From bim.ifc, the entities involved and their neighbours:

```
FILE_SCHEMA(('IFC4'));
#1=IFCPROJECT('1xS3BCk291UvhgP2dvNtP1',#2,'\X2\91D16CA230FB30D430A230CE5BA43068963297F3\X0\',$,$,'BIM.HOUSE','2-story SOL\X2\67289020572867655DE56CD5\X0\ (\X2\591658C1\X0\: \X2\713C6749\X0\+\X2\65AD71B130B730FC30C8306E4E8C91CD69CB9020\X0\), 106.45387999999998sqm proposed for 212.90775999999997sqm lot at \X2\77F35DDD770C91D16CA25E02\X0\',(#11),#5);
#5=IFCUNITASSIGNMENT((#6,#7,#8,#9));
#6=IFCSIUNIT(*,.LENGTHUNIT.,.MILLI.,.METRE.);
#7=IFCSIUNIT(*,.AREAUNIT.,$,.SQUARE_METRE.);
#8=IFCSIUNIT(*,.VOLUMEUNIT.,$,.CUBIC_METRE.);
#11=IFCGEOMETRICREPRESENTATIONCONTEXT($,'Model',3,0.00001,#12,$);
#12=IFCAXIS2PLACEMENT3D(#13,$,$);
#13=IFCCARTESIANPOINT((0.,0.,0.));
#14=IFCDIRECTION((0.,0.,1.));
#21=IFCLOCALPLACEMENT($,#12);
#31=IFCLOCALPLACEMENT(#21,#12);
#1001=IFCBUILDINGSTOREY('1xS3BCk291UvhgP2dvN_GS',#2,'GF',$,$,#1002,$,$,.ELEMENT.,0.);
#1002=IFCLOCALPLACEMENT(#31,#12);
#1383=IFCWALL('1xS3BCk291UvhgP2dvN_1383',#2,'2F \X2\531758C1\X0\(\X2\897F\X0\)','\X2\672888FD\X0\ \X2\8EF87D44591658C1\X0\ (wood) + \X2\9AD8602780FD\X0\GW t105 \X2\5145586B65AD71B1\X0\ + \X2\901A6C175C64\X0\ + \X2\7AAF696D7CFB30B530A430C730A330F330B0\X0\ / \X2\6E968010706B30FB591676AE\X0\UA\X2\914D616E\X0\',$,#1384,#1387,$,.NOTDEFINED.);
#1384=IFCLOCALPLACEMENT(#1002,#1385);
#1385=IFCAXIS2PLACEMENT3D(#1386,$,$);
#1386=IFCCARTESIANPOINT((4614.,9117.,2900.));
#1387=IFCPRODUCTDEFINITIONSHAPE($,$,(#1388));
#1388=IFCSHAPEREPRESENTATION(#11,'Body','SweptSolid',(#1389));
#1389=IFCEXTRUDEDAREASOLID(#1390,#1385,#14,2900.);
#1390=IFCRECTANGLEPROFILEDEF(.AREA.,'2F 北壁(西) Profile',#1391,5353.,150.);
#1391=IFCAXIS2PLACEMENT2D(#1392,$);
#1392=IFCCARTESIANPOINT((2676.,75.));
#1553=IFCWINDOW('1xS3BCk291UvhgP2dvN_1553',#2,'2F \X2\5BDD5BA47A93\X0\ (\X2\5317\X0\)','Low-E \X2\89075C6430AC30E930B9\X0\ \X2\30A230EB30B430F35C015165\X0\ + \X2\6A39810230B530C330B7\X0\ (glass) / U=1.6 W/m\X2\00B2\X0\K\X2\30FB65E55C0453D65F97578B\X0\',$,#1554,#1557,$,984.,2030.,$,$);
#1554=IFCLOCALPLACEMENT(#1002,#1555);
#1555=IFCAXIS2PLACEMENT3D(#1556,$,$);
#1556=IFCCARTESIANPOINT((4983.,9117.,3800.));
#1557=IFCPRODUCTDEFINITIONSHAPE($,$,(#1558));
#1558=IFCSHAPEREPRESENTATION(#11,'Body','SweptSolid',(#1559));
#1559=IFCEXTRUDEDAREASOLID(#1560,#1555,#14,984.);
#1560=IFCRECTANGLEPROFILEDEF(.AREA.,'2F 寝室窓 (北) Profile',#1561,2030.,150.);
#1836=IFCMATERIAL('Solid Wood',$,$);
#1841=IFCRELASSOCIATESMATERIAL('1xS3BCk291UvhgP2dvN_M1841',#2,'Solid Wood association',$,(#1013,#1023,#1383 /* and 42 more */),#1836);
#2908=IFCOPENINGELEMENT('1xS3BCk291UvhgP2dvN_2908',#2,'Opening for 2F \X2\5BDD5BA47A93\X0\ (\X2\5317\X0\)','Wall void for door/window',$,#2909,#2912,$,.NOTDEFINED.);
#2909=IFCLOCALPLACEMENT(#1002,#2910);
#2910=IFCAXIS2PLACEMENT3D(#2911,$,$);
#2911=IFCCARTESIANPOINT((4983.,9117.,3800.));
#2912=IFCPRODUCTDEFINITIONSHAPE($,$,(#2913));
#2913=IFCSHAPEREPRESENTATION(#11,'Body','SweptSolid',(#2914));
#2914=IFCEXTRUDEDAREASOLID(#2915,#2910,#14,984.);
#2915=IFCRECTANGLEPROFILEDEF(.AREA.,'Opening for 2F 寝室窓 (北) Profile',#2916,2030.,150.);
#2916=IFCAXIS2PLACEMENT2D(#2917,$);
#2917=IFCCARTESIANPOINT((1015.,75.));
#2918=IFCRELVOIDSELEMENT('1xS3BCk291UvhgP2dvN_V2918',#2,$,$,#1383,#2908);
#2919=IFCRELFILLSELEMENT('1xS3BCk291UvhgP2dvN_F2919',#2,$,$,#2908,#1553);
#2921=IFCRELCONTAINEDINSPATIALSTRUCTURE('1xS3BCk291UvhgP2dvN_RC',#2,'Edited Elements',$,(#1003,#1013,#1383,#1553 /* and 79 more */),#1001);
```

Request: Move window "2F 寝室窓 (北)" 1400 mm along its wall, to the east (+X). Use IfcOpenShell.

```python
import ifcopenshell
import ifcopenshell.api.geometry
import ifcopenshell.util.placement

model = ifcopenshell.open("bim.ifc")

window = model.by_guid("1xS3BCk291UvhgP2dvN_1553")
opening = window.FillsVoids[0].RelatingOpeningElement
wall = opening.VoidsElements[0].RelatingBuildingElement

wall_matrix = ifcopenshell.util.placement.get_local_placement(wall.ObjectPlacement)
shift = wall_matrix[:3, 0] * 1400.0
before = ifcopenshell.util.placement.get_local_placement(window.ObjectPlacement)[:3, 3].copy()

# The window is not placed relative to its opening, so move both.
for product in (opening, window):
    matrix = ifcopenshell.util.placement.get_local_placement(product.ObjectPlacement)
    matrix[:3, 3] += shift
    ifcopenshell.api.geometry.edit_object_placement(model, product=product, matrix=matrix, is_si=False)

after = ifcopenshell.util.placement.get_local_placement(window.ObjectPlacement)[:3, 3]
print("window moved by", (after - before).round(3) + 0.0)

model.write("bim_v2.ifc")
```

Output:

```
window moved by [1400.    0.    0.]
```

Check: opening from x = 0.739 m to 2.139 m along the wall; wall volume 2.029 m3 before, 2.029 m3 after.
